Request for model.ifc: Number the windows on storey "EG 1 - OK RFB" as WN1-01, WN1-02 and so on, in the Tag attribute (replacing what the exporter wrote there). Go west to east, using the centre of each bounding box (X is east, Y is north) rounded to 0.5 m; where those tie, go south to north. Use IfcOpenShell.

First a look at what the model holds.

```python
import ifcopenshell
import ifcopenshell.util.element
import ifcopenshell.util.placement

model = ifcopenshell.open("model.ifc")
print(model.schema)
storey = next(s for s in model.by_type("IfcBuildingStorey") if s.Name == "EG 1 - OK RFB")
windows = [e for e in ifcopenshell.util.element.get_decomposition(storey) if e.is_a("IfcWindow")]
for e in sorted(windows, key=lambda e: e.id()):
    origin = ifcopenshell.util.placement.get_local_placement(e.ObjectPlacement)[:3, 3]
    print(e.id(), e.Tag, e.Name, origin.round(2) + 0.0, sep=" | ")
```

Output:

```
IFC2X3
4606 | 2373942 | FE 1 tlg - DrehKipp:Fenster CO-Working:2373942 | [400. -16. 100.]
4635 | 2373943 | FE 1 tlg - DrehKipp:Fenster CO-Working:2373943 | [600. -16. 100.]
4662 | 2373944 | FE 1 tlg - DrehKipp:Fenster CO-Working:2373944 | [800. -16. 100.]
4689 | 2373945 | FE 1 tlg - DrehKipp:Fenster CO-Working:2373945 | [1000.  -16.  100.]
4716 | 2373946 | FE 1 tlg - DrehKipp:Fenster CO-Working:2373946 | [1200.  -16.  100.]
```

```python
import ifcopenshell
import ifcopenshell.geom
import ifcopenshell.util.element
import ifcopenshell.util.shape

model = ifcopenshell.open("model.ifc")
settings = ifcopenshell.geom.settings()
settings.set("use-world-coords", True)


def centre(element):
    shape = ifcopenshell.geom.create_shape(settings, element)
    return ifcopenshell.util.shape.get_bbox_centroid(shape.geometry)


storey = next(s for s in model.by_type("IfcBuildingStorey") if s.Name == "EG 1 - OK RFB")
windows = [e for e in ifcopenshell.util.element.get_decomposition(storey) if e.is_a("IfcWindow")]

# Insertion points can sit at a corner or the storey origin, so sort by the geometry (in metres).
centres = {e: centre(e) for e in windows}
windows.sort(key=lambda e: (round(centres[e][0] / 0.5), centres[e][1]))

for i, e in enumerate(windows, start=1):
    number = f"WN1-{i:02d}"
    e.Tag = number
    print(e.id(), number)

model.write("model-out.ifc")
```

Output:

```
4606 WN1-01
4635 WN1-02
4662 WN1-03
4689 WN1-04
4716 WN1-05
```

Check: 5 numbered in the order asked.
